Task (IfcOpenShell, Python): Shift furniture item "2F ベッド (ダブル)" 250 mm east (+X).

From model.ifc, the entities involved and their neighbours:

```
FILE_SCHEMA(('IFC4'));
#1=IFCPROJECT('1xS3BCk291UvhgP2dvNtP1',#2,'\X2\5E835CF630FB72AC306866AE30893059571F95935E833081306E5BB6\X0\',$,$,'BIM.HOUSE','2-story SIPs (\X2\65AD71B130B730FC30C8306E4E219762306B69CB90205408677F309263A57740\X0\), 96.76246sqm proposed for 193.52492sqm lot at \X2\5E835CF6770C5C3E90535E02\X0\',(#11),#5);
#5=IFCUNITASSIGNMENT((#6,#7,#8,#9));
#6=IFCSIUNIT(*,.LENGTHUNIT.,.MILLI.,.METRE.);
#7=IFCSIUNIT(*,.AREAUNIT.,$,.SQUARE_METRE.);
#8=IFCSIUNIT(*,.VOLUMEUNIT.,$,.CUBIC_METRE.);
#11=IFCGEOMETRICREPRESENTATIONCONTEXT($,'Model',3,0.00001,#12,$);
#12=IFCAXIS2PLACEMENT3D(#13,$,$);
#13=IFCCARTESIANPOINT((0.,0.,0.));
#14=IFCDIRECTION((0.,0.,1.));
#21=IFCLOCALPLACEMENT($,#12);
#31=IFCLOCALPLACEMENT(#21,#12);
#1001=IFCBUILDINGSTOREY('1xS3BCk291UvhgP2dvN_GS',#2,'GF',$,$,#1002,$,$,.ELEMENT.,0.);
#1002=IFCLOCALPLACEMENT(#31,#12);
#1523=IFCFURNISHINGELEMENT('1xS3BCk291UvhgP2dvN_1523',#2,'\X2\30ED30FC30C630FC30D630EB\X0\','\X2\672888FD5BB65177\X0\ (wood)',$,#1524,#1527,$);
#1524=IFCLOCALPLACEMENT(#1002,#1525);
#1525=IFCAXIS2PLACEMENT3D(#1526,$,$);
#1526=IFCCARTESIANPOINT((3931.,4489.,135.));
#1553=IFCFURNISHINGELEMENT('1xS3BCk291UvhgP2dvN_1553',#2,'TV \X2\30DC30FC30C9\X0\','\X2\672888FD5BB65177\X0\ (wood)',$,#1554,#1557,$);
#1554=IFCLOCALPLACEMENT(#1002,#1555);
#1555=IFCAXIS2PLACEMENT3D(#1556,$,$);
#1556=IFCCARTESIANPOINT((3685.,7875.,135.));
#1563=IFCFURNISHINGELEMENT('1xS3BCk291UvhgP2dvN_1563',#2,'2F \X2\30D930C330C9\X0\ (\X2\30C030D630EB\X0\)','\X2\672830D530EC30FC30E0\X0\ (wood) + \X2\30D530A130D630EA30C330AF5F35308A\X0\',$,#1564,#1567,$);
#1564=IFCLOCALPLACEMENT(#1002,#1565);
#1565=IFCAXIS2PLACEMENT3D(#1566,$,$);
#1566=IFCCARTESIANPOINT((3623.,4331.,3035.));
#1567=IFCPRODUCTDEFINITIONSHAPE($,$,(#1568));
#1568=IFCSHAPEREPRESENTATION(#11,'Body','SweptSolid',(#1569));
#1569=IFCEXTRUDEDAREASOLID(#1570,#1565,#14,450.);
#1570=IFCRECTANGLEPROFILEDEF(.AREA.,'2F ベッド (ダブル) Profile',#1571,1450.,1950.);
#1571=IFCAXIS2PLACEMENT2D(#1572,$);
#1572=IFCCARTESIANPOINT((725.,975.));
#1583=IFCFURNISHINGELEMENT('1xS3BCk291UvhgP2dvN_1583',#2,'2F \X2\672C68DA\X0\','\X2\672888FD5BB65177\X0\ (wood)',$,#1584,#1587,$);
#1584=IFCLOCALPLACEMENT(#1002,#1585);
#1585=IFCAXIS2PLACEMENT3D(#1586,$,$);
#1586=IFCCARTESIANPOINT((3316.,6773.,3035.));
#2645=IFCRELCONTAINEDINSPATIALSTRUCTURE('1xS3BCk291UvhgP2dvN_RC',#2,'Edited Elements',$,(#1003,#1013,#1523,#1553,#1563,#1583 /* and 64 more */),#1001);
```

```python
import ifcopenshell
import ifcopenshell.api.geometry
import ifcopenshell.util.placement
import ifcopenshell.util.unit

model = ifcopenshell.open("model.ifc")
unit_scale = ifcopenshell.util.unit.calculate_unit_scale(model)

item = model.by_guid("1xS3BCk291UvhgP2dvN_1563")
matrix = ifcopenshell.util.placement.get_local_placement(item.ObjectPlacement)
matrix[0, 3] += 0.25 / unit_scale
ifcopenshell.api.geometry.edit_object_placement(model, product=item, matrix=matrix, is_si=False)

print(ifcopenshell.util.placement.get_local_placement(item.ObjectPlacement).round(3) + 0.0)

model.write("model_updated.ifc")
```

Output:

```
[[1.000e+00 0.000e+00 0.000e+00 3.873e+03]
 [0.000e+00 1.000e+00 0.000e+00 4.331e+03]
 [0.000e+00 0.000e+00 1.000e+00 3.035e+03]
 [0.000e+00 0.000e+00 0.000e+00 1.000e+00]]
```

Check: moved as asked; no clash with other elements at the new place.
